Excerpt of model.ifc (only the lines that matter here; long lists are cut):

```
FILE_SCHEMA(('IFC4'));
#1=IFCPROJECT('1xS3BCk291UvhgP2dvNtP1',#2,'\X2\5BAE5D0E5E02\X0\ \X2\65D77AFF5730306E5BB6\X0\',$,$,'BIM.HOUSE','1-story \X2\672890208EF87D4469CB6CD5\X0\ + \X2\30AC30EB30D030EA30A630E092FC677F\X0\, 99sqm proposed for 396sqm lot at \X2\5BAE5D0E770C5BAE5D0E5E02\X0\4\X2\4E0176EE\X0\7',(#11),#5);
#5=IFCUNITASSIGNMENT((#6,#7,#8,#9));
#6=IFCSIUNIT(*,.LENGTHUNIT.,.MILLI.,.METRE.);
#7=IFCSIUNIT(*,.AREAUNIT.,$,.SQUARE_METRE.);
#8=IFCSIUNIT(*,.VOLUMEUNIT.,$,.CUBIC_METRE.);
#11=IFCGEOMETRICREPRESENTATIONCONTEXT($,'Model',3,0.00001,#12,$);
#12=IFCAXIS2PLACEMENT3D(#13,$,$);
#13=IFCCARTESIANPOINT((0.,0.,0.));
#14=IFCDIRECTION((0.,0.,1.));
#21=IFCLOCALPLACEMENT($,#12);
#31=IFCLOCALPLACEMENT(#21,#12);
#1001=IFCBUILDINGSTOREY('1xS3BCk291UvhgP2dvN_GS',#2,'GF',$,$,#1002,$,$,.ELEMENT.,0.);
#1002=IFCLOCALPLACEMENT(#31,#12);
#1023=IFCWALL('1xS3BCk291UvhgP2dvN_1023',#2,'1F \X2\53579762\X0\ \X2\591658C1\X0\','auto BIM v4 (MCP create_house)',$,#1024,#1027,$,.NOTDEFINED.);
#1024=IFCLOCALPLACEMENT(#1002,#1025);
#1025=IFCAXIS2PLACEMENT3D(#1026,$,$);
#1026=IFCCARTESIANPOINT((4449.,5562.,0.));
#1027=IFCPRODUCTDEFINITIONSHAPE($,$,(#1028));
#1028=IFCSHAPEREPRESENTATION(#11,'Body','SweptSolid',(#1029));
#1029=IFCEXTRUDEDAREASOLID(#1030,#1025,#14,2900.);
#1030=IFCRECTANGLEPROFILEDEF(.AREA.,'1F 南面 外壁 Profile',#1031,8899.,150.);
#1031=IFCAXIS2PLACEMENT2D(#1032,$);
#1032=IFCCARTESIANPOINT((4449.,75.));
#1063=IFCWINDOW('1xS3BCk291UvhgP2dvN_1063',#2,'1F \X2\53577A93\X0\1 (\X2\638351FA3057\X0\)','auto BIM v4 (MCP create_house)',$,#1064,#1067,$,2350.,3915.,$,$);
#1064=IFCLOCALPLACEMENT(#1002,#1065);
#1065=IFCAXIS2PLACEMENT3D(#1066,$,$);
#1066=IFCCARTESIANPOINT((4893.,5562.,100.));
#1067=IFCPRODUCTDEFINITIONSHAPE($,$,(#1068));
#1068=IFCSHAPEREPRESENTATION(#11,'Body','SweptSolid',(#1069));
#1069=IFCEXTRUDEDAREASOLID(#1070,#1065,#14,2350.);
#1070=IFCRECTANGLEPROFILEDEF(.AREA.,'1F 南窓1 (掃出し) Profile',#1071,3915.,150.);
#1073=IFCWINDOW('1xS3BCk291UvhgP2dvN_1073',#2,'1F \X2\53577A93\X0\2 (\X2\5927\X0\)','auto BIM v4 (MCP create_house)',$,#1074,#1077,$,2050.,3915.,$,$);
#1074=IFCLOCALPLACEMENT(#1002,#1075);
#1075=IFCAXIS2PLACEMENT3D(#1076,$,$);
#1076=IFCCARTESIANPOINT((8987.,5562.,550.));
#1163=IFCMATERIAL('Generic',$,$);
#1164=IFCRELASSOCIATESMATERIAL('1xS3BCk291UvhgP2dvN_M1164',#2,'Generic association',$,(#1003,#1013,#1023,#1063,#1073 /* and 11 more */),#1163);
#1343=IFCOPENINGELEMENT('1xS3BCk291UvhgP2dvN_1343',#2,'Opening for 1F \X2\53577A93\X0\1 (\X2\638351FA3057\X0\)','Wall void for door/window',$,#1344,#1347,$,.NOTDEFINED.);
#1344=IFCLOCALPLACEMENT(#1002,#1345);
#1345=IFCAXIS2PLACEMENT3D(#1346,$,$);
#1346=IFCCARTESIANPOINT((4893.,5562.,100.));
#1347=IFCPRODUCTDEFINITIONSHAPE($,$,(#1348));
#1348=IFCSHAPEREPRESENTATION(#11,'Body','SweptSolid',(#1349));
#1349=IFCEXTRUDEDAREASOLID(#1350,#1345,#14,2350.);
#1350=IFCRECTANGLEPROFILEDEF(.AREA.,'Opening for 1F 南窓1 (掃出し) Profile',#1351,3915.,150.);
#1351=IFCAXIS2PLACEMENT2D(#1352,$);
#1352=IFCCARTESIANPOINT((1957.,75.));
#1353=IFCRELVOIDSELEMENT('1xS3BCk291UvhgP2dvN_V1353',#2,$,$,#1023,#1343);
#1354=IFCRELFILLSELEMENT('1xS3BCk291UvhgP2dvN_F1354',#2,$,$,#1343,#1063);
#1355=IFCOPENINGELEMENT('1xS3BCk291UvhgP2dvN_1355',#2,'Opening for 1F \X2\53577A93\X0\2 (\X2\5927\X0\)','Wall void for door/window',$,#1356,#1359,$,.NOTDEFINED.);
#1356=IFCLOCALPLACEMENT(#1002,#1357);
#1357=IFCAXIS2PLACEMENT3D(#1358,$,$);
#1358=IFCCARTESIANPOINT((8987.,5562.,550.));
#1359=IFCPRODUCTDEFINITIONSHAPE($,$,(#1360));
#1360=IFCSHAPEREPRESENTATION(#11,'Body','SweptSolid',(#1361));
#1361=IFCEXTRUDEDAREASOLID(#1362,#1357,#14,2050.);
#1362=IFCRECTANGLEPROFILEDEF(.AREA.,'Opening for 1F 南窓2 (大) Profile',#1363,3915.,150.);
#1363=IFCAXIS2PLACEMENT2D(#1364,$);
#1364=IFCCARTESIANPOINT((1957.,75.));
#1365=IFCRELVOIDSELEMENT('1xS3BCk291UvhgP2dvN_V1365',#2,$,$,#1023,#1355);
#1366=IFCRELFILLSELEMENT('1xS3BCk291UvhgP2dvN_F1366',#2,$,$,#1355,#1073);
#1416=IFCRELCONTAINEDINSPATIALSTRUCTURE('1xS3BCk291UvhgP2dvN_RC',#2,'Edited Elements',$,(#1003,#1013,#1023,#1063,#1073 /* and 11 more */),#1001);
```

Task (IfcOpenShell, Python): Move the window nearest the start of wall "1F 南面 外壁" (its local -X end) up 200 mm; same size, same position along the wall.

```python
import numpy as np
import ifcopenshell
import ifcopenshell.api.geometry
import ifcopenshell.util.placement
import ifcopenshell.util.unit

model = ifcopenshell.open("model.ifc")
unit_scale = ifcopenshell.util.unit.calculate_unit_scale(model)

window = model.by_guid("1xS3BCk291UvhgP2dvN_1063")
opening = window.FillsVoids[0].RelatingOpeningElement
dz = 200.0

shift = np.array([0.0, 0.0, dz])
# The window is not placed relative to its opening, so move both.
for product in (opening, window):
    matrix = ifcopenshell.util.placement.get_local_placement(product.ObjectPlacement)
    matrix[:3, 3] += shift
    ifcopenshell.api.geometry.edit_object_placement(model, product=product, matrix=matrix, is_si=False)

print(f"moved by {dz * unit_scale:+.3f} m")

model.write("model_rev.ifc")
```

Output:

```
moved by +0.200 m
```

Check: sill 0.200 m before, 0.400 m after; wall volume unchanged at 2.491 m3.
